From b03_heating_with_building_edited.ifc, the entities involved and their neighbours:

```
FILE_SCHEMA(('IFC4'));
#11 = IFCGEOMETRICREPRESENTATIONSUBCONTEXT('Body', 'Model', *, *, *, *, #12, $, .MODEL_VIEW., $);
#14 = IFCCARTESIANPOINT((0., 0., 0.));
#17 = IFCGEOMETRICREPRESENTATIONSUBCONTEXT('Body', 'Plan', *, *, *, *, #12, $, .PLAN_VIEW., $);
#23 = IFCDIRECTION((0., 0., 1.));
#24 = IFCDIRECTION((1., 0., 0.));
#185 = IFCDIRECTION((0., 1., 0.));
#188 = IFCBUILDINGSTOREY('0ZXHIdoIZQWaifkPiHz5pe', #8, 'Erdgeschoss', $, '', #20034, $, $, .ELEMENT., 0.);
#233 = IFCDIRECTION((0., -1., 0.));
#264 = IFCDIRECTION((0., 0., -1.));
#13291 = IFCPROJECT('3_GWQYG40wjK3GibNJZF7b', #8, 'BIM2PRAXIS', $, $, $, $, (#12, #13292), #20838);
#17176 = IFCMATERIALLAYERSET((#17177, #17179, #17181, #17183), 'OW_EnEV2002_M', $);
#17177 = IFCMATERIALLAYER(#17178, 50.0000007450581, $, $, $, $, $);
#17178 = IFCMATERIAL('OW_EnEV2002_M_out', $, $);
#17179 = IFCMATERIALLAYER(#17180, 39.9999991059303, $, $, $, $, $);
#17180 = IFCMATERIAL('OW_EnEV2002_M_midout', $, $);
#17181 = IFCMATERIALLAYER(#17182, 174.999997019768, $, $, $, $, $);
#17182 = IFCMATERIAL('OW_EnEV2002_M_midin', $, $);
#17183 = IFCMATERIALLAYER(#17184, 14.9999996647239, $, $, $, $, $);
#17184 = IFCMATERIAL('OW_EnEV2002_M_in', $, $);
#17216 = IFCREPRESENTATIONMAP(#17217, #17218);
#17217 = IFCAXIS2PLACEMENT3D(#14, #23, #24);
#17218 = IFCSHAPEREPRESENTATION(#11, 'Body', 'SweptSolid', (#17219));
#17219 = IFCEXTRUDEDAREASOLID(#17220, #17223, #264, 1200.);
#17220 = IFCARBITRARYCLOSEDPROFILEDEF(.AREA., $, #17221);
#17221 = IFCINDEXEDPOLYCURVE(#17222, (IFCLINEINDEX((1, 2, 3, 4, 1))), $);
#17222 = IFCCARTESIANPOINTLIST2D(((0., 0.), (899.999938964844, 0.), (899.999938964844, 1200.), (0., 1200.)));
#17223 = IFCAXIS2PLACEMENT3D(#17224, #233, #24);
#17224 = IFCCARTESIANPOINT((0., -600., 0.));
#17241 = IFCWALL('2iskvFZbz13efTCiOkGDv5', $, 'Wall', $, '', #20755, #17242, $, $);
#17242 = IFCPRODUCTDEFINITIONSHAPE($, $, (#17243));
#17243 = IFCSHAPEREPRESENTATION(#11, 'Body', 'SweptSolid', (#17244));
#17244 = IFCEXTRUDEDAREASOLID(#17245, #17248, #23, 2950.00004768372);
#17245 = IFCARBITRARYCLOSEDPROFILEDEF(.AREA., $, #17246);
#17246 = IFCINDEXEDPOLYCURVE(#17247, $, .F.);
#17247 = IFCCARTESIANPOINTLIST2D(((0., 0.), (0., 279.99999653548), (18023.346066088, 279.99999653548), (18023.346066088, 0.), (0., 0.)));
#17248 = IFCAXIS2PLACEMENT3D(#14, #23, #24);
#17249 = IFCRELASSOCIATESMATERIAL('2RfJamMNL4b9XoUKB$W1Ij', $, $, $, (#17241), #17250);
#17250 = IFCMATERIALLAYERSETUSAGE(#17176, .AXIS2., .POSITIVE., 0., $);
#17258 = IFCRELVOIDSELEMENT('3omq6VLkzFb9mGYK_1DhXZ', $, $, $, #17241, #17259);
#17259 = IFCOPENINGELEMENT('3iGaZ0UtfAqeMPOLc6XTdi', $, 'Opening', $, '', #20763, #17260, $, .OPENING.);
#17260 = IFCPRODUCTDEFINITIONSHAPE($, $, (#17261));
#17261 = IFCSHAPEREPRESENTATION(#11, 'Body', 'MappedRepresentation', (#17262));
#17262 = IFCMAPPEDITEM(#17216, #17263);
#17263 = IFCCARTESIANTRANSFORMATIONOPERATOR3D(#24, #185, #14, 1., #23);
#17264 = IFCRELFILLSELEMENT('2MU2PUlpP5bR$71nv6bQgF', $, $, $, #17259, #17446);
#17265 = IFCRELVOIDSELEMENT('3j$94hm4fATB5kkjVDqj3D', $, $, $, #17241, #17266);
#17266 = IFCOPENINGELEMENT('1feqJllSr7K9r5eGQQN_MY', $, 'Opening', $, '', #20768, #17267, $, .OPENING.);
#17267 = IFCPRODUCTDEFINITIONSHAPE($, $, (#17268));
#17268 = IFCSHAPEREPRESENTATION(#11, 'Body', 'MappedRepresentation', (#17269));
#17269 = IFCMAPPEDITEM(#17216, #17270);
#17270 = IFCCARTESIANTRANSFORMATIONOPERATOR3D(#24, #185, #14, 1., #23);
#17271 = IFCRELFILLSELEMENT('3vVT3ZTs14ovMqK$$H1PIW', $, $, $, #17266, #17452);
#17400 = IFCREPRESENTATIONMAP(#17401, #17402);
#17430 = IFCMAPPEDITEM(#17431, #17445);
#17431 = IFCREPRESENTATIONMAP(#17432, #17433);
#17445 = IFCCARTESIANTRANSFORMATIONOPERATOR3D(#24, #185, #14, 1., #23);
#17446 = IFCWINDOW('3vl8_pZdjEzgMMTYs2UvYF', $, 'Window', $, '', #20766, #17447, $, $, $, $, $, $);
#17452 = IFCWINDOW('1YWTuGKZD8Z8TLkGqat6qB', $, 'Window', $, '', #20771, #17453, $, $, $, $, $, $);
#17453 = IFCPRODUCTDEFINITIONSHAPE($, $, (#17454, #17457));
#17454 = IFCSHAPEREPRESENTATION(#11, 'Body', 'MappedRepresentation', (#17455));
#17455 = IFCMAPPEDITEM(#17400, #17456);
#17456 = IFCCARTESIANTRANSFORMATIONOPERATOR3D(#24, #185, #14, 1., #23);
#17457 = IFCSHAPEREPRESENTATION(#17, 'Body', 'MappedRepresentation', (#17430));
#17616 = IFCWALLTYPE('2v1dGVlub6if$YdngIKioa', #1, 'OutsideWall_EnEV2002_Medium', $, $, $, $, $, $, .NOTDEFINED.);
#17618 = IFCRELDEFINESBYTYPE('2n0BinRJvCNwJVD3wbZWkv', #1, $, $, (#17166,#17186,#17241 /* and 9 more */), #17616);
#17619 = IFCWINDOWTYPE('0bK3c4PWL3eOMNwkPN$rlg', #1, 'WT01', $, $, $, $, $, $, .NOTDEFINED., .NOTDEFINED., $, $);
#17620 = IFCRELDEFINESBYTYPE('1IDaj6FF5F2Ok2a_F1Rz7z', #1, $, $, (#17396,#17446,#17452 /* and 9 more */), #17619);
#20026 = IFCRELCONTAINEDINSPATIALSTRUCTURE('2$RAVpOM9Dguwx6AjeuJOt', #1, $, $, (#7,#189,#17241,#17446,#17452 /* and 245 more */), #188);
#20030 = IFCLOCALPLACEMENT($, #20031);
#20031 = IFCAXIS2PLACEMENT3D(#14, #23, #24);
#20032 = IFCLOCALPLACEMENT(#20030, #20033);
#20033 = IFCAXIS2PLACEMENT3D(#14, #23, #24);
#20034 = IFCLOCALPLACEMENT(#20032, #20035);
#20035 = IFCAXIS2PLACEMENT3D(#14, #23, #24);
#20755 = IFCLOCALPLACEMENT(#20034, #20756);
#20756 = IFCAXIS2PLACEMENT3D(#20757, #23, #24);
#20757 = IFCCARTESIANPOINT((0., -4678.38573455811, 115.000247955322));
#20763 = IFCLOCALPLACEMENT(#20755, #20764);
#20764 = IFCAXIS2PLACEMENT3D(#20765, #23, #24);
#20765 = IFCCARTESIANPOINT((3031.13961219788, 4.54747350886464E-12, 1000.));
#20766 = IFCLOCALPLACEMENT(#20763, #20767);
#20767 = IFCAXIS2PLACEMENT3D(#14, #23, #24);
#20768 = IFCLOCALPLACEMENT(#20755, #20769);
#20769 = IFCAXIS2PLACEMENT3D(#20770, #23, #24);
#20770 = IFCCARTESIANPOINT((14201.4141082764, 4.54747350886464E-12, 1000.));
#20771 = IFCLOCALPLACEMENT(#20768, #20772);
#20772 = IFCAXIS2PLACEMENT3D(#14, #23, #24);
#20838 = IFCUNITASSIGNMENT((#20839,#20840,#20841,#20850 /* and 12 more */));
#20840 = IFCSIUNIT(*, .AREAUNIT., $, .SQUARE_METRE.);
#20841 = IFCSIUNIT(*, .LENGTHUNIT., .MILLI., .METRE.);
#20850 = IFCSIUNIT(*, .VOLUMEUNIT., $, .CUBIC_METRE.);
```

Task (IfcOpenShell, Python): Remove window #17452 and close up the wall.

```python
import ifcopenshell
import ifcopenshell.api.feature
import ifcopenshell.api.root
import ifcopenshell.geom
import ifcopenshell.util.shape

model = ifcopenshell.open("b03_heating_with_building_edited.ifc")
settings = ifcopenshell.geom.settings()


def volume(element):
    """Net volume in cubic metres, openings subtracted."""
    shape = ifcopenshell.geom.create_shape(settings, element)
    return ifcopenshell.util.shape.get_volume(shape.geometry)


window = model.by_guid("1YWTuGKZD8Z8TLkGqat6qB")
opening = window.FillsVoids[0].RelatingOpeningElement
wall = opening.VoidsElements[0].RelatingBuildingElement
before = volume(wall)

ifcopenshell.api.root.remove_product(model, product=window)
ifcopenshell.api.feature.remove_feature(model, feature=opening)

after = volume(wall)

print(f"wall volume {before:.3f} -> {after:.3f} m3")

model.write("b03_heating_with_building_edited_updated.ifc")
```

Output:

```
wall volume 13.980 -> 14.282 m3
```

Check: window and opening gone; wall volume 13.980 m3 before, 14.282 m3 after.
